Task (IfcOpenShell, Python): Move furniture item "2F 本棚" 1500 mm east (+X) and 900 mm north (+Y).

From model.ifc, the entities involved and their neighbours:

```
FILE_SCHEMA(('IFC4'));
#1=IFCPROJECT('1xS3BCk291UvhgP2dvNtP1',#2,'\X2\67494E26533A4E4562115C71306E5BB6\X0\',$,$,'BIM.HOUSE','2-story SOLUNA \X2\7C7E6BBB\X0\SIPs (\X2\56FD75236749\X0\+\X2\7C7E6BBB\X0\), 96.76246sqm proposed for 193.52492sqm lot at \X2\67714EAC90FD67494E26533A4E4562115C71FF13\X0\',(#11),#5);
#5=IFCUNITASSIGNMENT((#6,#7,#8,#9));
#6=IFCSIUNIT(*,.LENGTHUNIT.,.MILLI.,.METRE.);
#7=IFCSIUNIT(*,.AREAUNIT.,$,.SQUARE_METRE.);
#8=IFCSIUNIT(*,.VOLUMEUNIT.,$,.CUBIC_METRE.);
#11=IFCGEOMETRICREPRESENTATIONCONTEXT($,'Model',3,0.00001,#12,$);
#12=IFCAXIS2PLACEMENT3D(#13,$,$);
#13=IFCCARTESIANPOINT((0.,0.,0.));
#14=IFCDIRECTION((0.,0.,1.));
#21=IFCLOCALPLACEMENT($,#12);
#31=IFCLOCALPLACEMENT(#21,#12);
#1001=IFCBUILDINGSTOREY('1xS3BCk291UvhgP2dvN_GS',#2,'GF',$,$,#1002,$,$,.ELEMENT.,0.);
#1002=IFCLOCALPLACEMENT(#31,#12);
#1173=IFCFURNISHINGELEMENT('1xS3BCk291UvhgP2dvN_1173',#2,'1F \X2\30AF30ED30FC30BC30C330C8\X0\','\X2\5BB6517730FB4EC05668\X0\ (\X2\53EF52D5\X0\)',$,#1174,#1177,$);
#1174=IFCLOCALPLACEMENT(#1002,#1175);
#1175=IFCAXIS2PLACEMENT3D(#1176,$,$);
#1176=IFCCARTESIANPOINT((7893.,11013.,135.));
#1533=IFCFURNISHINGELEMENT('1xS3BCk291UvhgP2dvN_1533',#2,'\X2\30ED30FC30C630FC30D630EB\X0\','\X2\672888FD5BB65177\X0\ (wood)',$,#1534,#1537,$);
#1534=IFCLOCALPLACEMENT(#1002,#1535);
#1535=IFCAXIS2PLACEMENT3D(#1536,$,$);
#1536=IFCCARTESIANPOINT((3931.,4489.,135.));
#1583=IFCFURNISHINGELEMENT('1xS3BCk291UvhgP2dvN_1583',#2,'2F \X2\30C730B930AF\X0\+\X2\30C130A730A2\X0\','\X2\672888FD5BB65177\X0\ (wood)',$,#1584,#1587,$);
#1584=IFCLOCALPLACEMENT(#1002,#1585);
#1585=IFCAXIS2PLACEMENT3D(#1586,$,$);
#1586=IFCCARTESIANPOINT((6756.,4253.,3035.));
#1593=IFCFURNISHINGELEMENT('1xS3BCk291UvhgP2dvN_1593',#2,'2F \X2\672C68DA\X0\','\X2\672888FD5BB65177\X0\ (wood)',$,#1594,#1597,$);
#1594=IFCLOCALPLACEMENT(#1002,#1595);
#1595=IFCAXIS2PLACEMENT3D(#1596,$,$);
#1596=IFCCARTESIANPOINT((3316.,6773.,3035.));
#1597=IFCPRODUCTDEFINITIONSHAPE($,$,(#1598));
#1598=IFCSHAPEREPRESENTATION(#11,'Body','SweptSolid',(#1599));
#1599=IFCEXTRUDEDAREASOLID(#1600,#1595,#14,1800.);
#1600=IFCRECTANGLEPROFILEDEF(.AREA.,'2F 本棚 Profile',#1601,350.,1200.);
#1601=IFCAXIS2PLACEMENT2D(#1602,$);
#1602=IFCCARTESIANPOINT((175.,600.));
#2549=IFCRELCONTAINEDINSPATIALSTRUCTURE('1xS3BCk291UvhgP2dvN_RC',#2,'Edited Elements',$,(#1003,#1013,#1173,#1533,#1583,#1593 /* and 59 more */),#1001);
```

```python
import ifcopenshell
import ifcopenshell.api.geometry
import ifcopenshell.util.placement
import ifcopenshell.util.unit

model = ifcopenshell.open("model.ifc")
unit_scale = ifcopenshell.util.unit.calculate_unit_scale(model)

item = model.by_guid("1xS3BCk291UvhgP2dvN_1593")
matrix = ifcopenshell.util.placement.get_local_placement(item.ObjectPlacement)
matrix[0, 3] += 1.5 / unit_scale
matrix[1, 3] += 0.9 / unit_scale
ifcopenshell.api.geometry.edit_object_placement(model, product=item, matrix=matrix, is_si=False)

print(ifcopenshell.util.placement.get_local_placement(item.ObjectPlacement).round(3) + 0.0)

model.write("model_rev.ifc")
```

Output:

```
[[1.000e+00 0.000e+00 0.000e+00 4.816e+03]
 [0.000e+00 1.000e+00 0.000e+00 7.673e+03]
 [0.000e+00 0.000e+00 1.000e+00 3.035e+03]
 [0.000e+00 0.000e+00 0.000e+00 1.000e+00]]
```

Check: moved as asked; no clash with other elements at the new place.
